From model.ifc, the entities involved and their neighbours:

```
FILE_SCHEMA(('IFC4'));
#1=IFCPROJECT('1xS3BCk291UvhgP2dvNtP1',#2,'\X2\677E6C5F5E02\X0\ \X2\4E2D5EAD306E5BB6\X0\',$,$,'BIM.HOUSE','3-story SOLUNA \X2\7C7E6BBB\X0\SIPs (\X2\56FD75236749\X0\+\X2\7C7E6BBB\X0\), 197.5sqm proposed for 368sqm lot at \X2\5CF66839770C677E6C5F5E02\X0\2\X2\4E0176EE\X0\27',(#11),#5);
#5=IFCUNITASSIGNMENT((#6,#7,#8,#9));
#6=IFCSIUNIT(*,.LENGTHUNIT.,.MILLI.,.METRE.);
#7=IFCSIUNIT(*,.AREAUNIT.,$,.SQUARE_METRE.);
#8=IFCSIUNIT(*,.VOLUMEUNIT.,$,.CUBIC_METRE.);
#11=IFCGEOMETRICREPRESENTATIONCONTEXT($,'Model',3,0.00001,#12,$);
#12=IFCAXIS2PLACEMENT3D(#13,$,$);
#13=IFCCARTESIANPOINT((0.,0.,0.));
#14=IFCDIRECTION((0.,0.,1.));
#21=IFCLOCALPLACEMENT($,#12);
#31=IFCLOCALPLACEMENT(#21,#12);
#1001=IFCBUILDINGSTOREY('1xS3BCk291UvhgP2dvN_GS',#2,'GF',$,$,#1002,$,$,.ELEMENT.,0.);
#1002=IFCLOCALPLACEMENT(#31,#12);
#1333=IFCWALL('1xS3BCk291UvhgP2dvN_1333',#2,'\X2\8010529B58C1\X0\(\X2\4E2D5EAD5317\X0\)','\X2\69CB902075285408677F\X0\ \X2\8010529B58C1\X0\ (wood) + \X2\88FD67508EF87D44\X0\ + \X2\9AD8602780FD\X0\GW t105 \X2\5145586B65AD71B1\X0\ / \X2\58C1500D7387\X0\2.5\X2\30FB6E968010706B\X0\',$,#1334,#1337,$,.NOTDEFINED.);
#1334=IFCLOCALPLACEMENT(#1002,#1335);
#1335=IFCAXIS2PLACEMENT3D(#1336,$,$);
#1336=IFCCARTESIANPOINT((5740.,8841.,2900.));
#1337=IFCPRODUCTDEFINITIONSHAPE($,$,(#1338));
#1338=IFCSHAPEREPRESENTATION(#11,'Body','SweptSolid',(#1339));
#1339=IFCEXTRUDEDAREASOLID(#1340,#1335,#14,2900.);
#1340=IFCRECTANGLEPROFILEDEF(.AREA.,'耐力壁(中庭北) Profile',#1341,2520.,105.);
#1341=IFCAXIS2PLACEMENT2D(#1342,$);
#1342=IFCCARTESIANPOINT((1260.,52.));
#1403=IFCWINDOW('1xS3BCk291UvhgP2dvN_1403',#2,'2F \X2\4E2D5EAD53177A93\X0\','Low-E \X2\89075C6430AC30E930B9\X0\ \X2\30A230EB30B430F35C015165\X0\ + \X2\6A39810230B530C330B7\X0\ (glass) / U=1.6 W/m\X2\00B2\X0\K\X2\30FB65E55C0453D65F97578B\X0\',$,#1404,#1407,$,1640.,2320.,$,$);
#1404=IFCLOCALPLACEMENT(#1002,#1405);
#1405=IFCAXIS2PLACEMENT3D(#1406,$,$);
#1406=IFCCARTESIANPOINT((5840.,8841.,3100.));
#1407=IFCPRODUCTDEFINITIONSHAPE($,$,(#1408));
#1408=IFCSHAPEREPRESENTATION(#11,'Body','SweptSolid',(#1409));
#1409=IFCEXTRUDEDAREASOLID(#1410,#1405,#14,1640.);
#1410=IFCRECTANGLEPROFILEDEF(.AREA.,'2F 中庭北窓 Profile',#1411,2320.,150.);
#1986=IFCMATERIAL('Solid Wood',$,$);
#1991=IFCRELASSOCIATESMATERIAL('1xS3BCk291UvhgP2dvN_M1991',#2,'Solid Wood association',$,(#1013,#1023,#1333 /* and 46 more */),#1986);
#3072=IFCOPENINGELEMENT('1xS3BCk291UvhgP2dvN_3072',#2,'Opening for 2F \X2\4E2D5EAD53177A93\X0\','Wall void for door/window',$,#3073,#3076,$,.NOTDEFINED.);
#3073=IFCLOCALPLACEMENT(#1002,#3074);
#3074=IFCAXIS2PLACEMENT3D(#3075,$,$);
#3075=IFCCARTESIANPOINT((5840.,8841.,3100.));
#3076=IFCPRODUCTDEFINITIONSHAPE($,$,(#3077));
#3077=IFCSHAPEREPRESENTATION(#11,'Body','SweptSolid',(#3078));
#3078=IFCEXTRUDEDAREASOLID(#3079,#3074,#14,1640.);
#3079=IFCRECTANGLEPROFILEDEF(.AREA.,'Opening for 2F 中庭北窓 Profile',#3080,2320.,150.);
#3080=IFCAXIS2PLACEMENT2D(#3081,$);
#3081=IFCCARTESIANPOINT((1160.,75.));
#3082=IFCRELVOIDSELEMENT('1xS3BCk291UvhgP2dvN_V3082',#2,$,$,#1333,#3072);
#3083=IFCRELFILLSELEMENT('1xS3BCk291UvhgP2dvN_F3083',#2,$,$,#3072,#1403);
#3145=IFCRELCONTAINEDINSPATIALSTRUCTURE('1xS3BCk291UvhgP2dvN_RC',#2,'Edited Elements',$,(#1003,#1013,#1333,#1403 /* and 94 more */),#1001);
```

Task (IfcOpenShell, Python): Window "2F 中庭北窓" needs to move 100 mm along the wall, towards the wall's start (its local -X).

```python
import ifcopenshell
import ifcopenshell.api.geometry
import ifcopenshell.util.placement

model = ifcopenshell.open("model.ifc")

window = model.by_guid("1xS3BCk291UvhgP2dvN_1403")
opening = window.FillsVoids[0].RelatingOpeningElement
wall = opening.VoidsElements[0].RelatingBuildingElement

wall_matrix = ifcopenshell.util.placement.get_local_placement(wall.ObjectPlacement)
shift = wall_matrix[:3, 0] * -100.0
before = ifcopenshell.util.placement.get_local_placement(window.ObjectPlacement)[:3, 3].copy()

# The window is not placed relative to its opening, so move both.
for product in (opening, window):
    matrix = ifcopenshell.util.placement.get_local_placement(product.ObjectPlacement)
    matrix[:3, 3] += shift
    ifcopenshell.api.geometry.edit_object_placement(model, product=product, matrix=matrix, is_si=False)

after = ifcopenshell.util.placement.get_local_placement(window.ObjectPlacement)[:3, 3]
print("window moved by", (after - before).round(3) + 0.0)

model.write("model_edited.ifc")
```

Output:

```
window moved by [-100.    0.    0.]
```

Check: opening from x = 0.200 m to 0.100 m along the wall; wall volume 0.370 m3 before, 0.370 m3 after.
